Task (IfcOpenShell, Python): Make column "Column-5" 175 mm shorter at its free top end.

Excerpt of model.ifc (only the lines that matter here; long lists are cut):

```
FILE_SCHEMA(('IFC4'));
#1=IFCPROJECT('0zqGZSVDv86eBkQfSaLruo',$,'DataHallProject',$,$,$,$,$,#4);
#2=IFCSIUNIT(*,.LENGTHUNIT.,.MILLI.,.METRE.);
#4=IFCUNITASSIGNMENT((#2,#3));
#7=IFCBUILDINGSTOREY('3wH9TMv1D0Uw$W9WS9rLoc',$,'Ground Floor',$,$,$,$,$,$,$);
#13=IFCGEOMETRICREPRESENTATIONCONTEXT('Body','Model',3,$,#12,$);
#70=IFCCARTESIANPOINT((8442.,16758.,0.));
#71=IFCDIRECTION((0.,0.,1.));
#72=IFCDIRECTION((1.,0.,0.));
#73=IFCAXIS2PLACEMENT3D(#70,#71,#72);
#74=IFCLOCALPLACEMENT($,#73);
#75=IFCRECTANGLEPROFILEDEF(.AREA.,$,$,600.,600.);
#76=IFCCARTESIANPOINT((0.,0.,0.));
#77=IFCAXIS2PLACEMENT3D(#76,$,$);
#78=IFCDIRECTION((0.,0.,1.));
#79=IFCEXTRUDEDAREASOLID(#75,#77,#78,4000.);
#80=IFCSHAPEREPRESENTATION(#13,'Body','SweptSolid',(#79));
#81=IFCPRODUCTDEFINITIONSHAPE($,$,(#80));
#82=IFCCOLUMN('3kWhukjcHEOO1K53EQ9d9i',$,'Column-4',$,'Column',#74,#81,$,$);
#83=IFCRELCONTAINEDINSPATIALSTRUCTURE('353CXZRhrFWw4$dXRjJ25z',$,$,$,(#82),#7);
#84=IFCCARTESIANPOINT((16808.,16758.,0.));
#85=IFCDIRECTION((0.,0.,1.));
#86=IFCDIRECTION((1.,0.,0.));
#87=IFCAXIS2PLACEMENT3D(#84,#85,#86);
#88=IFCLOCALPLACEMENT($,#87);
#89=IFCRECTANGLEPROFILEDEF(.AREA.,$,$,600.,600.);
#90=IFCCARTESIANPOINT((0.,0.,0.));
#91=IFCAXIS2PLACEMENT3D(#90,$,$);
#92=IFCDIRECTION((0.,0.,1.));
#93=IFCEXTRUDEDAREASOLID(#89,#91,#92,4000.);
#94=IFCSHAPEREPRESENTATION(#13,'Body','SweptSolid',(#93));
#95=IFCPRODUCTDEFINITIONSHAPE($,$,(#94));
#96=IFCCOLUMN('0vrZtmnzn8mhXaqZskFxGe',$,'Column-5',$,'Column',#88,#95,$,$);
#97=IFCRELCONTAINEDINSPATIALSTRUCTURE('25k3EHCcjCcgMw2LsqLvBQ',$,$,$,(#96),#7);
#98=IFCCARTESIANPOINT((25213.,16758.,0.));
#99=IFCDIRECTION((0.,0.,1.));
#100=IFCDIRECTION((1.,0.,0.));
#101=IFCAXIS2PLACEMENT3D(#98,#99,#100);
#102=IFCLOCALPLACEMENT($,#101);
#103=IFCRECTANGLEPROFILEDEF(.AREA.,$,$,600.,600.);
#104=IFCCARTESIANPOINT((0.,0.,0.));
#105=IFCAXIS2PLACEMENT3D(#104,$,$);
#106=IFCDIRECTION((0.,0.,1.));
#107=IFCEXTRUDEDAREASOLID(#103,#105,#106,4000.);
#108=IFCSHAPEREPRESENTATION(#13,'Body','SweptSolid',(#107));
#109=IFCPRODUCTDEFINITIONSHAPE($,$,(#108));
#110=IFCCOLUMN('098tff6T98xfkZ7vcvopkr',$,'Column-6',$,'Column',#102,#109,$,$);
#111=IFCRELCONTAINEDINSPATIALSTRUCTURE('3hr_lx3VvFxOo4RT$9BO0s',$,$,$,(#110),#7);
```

```python
import ifcopenshell
import ifcopenshell.util.unit

model = ifcopenshell.open("model.ifc")
unit_scale = ifcopenshell.util.unit.calculate_unit_scale(model)

member = model.by_guid("0vrZtmnzn8mhXaqZskFxGe")
change = -0.175 / unit_scale

# The extrusion runs towards the end named, so only its depth changes.
body = next(r for r in member.Representation.Representations if r.RepresentationIdentifier == "Body")
solid = body.Items[0]
old_length = solid.Depth
solid.Depth += change

print(f"length {old_length:g} -> {solid.Depth:g}")

model.write("model_edited.ifc")
```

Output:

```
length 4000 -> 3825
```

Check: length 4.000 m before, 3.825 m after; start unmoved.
